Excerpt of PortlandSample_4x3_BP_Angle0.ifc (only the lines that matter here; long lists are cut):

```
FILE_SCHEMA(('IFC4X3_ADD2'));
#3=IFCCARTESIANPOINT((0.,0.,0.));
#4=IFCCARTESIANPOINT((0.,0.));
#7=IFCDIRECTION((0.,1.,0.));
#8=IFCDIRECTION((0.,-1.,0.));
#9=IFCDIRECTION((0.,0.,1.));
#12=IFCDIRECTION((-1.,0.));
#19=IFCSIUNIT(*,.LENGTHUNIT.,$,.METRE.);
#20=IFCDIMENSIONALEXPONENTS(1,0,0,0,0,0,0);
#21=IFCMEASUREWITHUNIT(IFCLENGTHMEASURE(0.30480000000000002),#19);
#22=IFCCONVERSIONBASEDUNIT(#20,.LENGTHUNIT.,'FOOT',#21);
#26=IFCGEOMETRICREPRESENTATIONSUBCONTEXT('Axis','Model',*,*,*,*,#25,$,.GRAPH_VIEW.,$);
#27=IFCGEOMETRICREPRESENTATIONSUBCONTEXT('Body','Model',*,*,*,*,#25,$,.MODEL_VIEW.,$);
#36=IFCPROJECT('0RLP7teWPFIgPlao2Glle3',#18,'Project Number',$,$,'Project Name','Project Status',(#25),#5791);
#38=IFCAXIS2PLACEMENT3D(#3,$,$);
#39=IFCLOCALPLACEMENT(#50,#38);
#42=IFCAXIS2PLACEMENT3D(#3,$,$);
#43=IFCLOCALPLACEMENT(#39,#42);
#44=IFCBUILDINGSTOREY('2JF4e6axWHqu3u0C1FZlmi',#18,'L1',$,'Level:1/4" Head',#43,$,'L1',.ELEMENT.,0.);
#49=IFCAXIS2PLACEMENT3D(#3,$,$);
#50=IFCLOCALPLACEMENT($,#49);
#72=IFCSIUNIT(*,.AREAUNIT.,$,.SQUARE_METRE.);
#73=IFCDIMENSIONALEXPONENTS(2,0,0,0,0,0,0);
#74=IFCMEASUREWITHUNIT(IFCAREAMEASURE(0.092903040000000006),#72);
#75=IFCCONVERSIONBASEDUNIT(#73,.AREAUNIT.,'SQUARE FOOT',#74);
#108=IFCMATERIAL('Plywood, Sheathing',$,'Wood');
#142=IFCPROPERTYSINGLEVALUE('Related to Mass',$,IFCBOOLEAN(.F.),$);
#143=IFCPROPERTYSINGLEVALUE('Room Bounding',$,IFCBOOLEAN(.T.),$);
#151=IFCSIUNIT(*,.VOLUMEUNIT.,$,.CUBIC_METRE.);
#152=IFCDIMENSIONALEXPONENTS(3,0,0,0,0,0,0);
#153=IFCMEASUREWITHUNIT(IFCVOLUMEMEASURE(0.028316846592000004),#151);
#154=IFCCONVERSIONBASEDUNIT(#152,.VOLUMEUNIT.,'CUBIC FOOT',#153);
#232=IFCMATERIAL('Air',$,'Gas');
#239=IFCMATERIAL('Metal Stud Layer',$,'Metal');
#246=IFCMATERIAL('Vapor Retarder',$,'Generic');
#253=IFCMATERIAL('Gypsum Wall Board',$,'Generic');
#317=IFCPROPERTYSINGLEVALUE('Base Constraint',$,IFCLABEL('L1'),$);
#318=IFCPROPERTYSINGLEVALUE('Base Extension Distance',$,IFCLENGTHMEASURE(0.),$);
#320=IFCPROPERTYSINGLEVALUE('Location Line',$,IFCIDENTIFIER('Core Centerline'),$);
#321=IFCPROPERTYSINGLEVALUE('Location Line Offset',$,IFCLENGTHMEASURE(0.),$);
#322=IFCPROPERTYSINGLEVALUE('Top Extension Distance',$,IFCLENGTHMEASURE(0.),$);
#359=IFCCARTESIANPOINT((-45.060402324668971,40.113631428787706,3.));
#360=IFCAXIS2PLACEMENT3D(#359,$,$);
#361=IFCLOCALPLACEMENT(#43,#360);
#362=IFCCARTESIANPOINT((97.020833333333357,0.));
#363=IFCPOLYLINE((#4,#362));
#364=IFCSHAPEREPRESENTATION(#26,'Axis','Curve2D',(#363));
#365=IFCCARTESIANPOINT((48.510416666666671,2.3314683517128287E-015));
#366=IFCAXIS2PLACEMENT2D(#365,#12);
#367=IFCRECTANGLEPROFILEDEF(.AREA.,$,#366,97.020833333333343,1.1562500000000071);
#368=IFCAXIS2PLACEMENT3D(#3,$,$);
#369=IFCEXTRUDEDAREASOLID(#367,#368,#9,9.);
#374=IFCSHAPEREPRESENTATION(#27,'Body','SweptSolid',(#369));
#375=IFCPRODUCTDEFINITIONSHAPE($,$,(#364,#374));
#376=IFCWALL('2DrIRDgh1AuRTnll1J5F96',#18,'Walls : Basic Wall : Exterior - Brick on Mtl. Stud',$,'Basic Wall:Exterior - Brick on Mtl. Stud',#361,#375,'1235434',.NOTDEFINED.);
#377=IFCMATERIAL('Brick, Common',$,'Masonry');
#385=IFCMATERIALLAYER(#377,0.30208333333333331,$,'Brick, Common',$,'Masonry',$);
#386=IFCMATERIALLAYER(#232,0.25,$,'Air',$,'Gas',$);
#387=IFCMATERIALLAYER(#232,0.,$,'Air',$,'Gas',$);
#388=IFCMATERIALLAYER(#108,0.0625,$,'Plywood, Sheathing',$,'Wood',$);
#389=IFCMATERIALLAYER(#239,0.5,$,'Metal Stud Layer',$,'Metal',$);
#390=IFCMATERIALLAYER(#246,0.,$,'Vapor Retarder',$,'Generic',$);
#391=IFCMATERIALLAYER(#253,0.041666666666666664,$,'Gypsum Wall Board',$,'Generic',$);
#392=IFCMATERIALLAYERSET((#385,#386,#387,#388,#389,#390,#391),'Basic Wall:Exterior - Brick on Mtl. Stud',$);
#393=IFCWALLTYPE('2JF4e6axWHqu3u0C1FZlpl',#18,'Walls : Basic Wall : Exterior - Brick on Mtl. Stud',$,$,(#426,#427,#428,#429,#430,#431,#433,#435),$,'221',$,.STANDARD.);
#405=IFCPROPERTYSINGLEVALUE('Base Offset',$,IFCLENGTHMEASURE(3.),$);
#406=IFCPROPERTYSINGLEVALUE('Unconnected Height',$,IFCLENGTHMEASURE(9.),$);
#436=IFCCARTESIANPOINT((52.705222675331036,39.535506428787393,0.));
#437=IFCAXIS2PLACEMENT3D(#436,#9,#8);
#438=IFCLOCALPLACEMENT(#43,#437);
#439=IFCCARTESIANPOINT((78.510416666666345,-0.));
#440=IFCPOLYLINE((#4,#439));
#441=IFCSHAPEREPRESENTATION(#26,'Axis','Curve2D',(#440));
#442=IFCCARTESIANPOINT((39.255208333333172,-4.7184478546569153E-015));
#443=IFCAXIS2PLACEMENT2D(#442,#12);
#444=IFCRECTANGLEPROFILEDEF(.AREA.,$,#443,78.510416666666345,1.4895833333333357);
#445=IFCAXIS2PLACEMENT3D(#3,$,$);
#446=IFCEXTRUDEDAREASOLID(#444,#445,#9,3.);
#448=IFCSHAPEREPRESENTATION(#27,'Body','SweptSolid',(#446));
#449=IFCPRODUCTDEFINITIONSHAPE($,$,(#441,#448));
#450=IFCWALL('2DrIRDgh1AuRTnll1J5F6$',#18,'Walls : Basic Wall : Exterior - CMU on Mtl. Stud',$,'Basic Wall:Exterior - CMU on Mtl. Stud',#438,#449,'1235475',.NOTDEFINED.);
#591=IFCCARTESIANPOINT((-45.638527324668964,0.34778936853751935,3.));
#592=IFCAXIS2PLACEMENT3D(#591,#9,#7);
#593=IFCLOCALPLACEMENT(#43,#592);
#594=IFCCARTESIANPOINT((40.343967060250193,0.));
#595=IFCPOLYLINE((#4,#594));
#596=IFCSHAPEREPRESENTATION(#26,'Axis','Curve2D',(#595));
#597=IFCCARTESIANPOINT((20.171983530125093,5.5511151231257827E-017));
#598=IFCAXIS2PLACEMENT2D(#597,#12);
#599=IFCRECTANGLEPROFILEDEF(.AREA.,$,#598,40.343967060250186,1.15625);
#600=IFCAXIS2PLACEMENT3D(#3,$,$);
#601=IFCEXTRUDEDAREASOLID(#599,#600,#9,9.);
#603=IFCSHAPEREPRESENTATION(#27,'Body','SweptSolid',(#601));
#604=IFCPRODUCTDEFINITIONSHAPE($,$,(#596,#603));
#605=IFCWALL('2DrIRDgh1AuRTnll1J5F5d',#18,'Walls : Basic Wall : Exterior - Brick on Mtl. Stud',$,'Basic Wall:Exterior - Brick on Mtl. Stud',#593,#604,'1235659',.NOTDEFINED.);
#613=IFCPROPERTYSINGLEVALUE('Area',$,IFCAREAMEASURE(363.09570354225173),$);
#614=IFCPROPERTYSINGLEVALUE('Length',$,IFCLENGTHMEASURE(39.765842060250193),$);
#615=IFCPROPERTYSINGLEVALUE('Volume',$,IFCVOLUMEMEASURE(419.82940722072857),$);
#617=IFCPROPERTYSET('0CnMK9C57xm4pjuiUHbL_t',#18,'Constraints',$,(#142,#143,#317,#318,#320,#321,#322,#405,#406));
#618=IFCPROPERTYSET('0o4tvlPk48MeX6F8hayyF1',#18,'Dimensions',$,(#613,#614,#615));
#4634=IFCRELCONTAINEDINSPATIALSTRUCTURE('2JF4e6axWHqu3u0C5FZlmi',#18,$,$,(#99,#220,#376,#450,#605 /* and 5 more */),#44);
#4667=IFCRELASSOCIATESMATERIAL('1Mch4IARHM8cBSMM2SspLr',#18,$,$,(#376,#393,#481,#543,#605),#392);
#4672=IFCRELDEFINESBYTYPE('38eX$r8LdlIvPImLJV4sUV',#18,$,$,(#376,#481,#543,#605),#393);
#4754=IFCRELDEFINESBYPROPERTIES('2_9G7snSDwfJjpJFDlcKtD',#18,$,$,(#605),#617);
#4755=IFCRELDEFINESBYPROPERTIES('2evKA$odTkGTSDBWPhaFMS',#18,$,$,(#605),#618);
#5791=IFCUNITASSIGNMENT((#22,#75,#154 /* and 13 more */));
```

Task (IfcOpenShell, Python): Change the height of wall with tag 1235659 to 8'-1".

```python
import ifcopenshell
import ifcopenshell.api.pset
import ifcopenshell.geom
import ifcopenshell.util.element
import ifcopenshell.util.representation
import ifcopenshell.util.shape
import ifcopenshell.util.unit

model = ifcopenshell.open("PortlandSample_4x3_BP_Angle0.ifc")
unit_scale = ifcopenshell.util.unit.calculate_unit_scale(model)
area_scale = ifcopenshell.util.unit.calculate_unit_scale(model, "AREAUNIT")
volume_scale = ifcopenshell.util.unit.calculate_unit_scale(model, "VOLUMEUNIT")
settings = ifcopenshell.geom.settings()


def volume(element):
    """Net volume in cubic metres, openings subtracted."""
    shape = ifcopenshell.geom.create_shape(settings, element)
    return ifcopenshell.util.shape.get_volume(shape.geometry)


wall = model.by_guid("2DrIRDgh1AuRTnll1J5F5d")
before = volume(wall)

body = ifcopenshell.util.representation.get_representation(wall, "Model", "Body")
solid = body.Items[0]
old_height = solid.Depth
solid.Depth = 97 * 0.0254 / unit_scale
after = volume(wall)
thickness = 0.3524  # wall thickness in metres

# Update the stored height, areas and volumes.
pset = model.by_id(ifcopenshell.util.element.get_pset(wall, "Constraints", should_inherit=False)["id"])
ifcopenshell.api.pset.edit_pset(model, pset=pset, properties={
    "Unconnected Height": model.create_entity("IfcLengthMeasure", solid.Depth),
})
pset = model.by_id(ifcopenshell.util.element.get_pset(wall, "Dimensions", should_inherit=False)["id"])
ifcopenshell.api.pset.edit_pset(model, pset=pset, properties={
    "Area": model.create_entity("IfcAreaMeasure", after / thickness / area_scale),
    "Volume": model.create_entity("IfcVolumeMeasure", after / volume_scale),
})

print(f"height {old_height:g} -> {solid.Depth:g}, volume {before:.3f} -> {after:.3f} m3")

model.write("PortlandSample_4x3_BP_Angle0_edited.ifc")
```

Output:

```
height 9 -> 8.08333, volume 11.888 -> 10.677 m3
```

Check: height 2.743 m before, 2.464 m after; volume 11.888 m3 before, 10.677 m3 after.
